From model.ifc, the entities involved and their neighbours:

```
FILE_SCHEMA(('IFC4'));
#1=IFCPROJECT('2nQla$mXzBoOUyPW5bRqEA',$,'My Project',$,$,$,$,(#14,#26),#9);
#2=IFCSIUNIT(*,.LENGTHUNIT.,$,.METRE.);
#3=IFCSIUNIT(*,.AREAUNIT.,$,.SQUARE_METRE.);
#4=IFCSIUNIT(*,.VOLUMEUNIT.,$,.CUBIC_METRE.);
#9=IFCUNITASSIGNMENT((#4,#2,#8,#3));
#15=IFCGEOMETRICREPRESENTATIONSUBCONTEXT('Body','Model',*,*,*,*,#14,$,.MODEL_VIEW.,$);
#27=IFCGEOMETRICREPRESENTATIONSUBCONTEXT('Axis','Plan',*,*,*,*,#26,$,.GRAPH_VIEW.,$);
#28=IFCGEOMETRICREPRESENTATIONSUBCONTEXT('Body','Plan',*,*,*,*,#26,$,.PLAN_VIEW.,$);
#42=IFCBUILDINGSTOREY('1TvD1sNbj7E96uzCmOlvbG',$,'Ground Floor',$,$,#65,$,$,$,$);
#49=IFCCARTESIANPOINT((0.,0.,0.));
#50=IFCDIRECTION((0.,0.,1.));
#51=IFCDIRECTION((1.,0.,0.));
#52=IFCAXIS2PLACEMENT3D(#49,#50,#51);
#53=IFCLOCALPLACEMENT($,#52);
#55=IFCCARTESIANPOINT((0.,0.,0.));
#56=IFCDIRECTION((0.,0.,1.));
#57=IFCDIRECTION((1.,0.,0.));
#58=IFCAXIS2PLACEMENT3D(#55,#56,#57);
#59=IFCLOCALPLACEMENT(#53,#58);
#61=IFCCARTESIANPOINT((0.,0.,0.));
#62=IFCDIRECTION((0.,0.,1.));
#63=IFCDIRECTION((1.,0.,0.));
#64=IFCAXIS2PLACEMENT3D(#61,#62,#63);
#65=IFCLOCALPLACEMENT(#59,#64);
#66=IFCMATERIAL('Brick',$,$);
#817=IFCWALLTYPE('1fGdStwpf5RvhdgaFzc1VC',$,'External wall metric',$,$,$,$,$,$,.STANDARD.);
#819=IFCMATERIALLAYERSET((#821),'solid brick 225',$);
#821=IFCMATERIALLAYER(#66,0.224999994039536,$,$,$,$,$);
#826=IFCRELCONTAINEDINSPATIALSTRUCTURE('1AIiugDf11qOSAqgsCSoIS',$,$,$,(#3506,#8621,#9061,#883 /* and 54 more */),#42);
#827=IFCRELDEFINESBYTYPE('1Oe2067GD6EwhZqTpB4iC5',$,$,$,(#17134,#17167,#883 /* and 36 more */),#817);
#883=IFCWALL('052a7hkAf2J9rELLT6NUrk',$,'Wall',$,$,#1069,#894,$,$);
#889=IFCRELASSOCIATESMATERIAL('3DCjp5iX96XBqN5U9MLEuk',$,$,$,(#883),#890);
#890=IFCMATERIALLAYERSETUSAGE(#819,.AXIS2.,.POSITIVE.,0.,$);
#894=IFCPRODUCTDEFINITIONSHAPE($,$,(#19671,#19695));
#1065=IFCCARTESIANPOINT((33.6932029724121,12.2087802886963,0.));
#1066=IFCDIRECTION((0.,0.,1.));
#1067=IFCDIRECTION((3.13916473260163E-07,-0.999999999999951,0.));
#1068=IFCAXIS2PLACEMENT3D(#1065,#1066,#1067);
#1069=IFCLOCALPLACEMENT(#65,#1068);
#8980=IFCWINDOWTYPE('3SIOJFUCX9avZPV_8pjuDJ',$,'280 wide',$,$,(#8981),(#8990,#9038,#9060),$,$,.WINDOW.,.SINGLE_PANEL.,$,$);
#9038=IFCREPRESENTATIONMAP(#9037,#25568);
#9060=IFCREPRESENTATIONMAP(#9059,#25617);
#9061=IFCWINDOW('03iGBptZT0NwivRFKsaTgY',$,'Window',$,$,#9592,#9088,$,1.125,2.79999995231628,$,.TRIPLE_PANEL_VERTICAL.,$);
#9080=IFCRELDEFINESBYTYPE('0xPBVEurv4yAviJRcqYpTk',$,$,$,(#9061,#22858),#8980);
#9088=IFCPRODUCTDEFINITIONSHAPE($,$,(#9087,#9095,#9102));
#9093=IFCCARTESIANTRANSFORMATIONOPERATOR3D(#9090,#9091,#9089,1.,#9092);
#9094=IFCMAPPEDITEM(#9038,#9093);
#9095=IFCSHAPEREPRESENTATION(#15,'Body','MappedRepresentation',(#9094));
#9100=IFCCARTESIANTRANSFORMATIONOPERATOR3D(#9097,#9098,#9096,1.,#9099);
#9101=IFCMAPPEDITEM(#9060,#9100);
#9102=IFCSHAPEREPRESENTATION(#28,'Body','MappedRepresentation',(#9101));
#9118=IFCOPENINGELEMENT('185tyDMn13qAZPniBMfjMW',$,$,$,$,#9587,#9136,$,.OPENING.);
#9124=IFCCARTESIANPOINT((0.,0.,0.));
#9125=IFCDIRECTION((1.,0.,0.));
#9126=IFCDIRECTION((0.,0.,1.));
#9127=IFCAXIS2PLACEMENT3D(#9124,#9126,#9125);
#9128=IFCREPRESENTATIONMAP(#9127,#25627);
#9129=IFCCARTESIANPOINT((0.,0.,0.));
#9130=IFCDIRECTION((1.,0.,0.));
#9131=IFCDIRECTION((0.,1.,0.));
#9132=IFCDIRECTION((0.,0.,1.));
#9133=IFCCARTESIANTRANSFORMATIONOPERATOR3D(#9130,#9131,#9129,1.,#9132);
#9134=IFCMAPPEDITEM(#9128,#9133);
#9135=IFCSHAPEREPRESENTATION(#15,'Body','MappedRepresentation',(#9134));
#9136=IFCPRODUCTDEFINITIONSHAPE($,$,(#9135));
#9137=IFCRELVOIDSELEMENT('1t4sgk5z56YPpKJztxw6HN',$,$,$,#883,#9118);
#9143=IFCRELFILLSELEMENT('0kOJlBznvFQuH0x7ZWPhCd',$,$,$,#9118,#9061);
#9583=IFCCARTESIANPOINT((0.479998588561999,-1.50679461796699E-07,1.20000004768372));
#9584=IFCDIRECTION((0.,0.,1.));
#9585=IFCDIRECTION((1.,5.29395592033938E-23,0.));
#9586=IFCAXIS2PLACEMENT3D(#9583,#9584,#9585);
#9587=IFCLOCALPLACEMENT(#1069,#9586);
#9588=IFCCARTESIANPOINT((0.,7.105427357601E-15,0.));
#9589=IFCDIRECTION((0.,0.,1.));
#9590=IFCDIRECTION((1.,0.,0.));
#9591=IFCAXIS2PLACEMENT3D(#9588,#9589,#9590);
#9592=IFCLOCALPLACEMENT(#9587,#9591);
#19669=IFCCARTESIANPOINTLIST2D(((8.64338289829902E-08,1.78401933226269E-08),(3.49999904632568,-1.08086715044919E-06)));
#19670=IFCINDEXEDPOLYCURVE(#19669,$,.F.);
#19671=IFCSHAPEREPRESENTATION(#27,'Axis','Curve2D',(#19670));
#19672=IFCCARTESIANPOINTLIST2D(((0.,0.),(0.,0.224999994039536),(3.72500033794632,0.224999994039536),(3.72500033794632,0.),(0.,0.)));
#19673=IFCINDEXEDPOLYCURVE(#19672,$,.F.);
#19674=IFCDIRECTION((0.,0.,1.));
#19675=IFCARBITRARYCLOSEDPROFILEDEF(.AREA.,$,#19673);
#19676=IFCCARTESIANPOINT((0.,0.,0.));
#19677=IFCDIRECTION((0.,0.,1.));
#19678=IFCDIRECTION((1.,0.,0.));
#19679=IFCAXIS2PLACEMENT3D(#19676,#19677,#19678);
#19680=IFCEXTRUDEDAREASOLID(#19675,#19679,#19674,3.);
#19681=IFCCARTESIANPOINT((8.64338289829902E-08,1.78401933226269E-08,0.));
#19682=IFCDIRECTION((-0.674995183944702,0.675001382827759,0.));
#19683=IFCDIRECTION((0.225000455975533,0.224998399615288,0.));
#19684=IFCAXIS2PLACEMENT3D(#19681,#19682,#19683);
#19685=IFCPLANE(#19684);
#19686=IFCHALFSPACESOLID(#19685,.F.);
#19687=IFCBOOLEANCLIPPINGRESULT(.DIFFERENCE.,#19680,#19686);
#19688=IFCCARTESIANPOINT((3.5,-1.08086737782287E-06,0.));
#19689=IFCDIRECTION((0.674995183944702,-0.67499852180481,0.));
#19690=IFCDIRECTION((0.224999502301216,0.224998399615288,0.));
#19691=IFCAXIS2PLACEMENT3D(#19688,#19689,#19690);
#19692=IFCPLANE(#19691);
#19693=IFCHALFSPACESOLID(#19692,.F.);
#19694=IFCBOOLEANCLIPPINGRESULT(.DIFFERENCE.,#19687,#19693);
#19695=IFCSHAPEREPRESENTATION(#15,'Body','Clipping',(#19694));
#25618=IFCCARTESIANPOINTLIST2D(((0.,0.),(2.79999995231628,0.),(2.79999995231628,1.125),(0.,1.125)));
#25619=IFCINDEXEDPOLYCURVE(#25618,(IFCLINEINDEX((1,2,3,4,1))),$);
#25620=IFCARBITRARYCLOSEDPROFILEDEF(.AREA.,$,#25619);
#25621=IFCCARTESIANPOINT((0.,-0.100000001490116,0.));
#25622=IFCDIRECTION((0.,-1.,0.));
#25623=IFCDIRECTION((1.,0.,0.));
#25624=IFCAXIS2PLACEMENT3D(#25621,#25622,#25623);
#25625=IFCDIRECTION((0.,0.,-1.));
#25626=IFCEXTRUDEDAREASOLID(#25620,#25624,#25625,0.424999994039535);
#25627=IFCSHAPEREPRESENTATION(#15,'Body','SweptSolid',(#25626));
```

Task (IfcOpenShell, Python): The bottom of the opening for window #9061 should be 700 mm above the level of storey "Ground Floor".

```python
import numpy as np
import ifcopenshell
import ifcopenshell.api.geometry
import ifcopenshell.geom
import ifcopenshell.util.element
import ifcopenshell.util.placement
import ifcopenshell.util.shape
import ifcopenshell.util.unit

model = ifcopenshell.open("model.ifc")
unit_scale = ifcopenshell.util.unit.calculate_unit_scale(model)

window = model.by_guid("03iGBptZT0NwivRFKsaTgY")
opening = window.FillsVoids[0].RelatingOpeningElement
storey = ifcopenshell.util.element.get_container(window, ifc_class="IfcBuildingStorey")
level = ifcopenshell.util.placement.get_local_placement(storey.ObjectPlacement)[2, 3]

# The opening's origin need not be at the sill, so measure its lowest point.
shape = ifcopenshell.geom.create_shape(ifcopenshell.geom.settings(), opening)
bottom = ifcopenshell.util.shape.get_shape_bottom_elevation(shape, shape.geometry) / unit_scale
dz = level + 0.7 / unit_scale - bottom

shift = np.array([0.0, 0.0, dz])
# The window is placed relative to its opening, so it follows when the opening moves.
matrix = ifcopenshell.util.placement.get_local_placement(opening.ObjectPlacement)
matrix[:3, 3] += shift
ifcopenshell.api.geometry.edit_object_placement(
    model, product=opening, matrix=matrix, is_si=False, should_transform_children=True
)

print(f"moved by {dz * unit_scale:+.3f} m")

model.write("model_rev.ifc")
```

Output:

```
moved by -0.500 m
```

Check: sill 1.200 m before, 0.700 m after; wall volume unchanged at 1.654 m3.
